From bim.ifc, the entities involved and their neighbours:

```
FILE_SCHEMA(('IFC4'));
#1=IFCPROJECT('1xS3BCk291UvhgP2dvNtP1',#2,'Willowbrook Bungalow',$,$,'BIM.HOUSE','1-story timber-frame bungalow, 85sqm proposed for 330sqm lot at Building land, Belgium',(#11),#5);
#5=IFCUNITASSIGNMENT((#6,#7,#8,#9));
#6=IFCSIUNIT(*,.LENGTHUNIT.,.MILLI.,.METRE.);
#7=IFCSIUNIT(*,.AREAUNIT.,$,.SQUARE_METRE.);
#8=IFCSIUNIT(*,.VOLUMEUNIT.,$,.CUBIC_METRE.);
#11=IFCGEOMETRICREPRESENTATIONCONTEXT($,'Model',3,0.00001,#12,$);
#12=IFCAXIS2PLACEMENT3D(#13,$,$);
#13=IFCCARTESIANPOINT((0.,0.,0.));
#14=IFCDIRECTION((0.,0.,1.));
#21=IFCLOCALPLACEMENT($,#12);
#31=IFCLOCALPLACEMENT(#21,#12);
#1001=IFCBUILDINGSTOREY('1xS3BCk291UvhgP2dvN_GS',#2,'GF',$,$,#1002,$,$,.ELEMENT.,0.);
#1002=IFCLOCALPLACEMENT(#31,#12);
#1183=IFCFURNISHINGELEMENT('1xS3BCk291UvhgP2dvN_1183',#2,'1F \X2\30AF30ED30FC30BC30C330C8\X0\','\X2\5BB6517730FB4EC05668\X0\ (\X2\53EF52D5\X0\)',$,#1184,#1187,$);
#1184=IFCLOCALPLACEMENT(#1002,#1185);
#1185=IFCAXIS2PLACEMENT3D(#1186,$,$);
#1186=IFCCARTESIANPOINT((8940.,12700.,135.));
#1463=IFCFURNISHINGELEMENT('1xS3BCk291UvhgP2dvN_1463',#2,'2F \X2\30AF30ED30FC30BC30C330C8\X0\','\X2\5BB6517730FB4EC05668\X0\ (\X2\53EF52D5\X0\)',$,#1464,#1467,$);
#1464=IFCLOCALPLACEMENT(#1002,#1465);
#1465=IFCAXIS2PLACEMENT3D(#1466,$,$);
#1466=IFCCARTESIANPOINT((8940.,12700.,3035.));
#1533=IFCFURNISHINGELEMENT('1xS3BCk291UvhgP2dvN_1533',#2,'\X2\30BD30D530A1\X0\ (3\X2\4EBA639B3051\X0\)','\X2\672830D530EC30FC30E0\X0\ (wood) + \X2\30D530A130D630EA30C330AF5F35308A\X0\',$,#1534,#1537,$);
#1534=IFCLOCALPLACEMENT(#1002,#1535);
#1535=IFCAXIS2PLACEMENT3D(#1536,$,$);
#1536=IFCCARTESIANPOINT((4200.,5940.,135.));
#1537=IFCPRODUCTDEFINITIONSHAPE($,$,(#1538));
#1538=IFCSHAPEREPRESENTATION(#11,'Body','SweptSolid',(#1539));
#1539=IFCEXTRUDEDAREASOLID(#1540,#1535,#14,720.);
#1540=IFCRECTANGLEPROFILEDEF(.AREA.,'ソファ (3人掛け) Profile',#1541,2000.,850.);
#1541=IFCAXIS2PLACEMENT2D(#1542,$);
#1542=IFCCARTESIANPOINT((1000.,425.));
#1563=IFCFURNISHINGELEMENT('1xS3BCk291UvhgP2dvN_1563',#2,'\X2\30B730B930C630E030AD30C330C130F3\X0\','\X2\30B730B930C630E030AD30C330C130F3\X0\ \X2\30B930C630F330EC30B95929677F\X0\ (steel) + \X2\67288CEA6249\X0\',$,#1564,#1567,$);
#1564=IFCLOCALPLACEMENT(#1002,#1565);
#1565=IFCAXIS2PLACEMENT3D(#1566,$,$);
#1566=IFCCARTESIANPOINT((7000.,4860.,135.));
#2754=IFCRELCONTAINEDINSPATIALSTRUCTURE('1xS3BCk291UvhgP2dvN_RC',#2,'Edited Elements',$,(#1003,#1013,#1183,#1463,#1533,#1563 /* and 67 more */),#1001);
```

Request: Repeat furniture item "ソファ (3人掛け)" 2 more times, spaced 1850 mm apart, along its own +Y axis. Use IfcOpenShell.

```python
import ifcopenshell
import ifcopenshell.api.geometry
import ifcopenshell.api.root
import ifcopenshell.util.element
import ifcopenshell.util.placement

model = ifcopenshell.open("bim.ifc")


def reuse_history(source, copy):
    """copy_class also copies each property set's owner history, people and application; keep the originals."""
    for rel in copy.IsDefinedBy:
        if rel.is_a("IfcRelDefinesByProperties") and (history := rel.RelatingPropertyDefinition.OwnerHistory):
            rel.RelatingPropertyDefinition.OwnerHistory = source.OwnerHistory
            ifcopenshell.util.element.remove_deep2(model, history)


source = model.by_guid("1xS3BCk291UvhgP2dvN_1533")
base = ifcopenshell.util.placement.get_local_placement(source.ObjectPlacement)
step = base[:3, 1] * 1850.0

for i in range(1, 3):
    copy = ifcopenshell.api.root.copy_class(model, product=source)
    copy.Representation = ifcopenshell.util.element.copy_deep(
        model, source.Representation, exclude=["IfcGeometricRepresentationContext", "IfcRepresentationMap"]
    )
    reuse_history(source, copy)
    matrix = base.copy()
    matrix[:3, 3] += i * step
    print("added at", matrix[:3, 3].round(3) + 0.0)
    ifcopenshell.api.geometry.edit_object_placement(model, product=copy, matrix=matrix, is_si=False)

model.write("bim_edited.ifc")
```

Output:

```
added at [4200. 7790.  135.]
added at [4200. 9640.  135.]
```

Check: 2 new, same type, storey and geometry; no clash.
